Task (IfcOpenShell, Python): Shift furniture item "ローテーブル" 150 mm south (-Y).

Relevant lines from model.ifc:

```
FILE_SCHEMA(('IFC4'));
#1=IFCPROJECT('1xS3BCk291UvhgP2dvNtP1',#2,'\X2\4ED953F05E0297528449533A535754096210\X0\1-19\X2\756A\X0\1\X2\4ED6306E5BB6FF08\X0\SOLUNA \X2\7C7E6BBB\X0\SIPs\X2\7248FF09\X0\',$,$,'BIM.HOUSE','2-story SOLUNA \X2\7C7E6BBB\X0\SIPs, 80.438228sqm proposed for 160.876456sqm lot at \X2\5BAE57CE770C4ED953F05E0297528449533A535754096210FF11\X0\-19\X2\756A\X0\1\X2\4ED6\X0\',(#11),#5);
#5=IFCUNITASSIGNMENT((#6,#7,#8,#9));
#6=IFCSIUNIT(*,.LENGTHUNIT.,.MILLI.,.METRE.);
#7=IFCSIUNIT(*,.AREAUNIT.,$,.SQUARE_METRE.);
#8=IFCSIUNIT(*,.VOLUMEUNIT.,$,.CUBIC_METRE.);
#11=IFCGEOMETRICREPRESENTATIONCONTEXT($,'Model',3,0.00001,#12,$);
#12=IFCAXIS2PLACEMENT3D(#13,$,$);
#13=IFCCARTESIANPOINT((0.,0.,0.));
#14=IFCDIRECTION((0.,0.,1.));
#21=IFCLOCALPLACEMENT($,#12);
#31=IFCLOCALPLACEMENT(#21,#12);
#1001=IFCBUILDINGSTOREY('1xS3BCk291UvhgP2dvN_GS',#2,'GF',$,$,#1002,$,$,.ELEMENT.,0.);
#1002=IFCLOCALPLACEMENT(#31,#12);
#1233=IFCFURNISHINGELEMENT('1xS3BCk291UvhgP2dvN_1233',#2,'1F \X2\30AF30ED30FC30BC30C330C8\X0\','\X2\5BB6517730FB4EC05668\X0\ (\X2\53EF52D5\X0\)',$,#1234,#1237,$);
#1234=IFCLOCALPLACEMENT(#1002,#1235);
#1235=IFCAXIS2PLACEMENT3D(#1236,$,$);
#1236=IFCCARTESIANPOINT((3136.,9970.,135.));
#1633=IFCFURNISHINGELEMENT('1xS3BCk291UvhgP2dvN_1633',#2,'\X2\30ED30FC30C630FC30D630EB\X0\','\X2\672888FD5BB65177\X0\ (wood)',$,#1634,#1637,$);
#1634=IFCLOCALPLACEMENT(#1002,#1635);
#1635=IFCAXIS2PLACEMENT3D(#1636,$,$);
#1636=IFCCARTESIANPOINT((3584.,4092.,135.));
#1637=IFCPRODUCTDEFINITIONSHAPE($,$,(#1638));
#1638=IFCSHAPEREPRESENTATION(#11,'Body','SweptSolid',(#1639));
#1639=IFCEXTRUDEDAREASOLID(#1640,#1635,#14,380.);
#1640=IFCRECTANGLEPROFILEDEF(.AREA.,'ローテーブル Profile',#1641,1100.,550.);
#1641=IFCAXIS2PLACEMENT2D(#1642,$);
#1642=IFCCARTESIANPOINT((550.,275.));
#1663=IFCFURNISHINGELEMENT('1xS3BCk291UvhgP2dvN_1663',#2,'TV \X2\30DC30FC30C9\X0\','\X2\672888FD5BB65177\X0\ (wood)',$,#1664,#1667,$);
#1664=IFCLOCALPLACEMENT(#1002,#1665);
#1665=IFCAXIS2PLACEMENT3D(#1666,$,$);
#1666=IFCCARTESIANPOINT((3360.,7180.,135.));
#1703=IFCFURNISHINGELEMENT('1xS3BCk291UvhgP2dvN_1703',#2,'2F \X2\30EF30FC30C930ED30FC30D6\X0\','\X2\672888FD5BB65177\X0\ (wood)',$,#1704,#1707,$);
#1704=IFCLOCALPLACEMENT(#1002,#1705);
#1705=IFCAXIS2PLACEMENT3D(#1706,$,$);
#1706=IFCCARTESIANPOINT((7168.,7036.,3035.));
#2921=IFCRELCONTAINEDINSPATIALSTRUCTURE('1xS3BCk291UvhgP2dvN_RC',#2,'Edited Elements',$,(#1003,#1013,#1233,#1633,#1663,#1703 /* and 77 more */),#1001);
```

```python
import ifcopenshell
import ifcopenshell.api.geometry
import ifcopenshell.util.placement

model = ifcopenshell.open("model.ifc")

item = model.by_guid("1xS3BCk291UvhgP2dvN_1633")
matrix = ifcopenshell.util.placement.get_local_placement(item.ObjectPlacement)
matrix[1, 3] -= 150.0
ifcopenshell.api.geometry.edit_object_placement(model, product=item, matrix=matrix, is_si=False)

print(ifcopenshell.util.placement.get_local_placement(item.ObjectPlacement).round(3) + 0.0)

model.write("model_v2.ifc")
```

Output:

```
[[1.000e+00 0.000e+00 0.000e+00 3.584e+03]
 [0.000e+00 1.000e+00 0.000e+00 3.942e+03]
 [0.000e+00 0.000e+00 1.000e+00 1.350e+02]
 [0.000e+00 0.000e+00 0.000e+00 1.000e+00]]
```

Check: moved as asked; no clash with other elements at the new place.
